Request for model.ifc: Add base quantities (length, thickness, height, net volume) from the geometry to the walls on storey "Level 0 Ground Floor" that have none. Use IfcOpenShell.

First a look at what the model holds.

```python
import ifcopenshell
import ifcopenshell.util.element
import ifcopenshell.util.unit

model = ifcopenshell.open("model.ifc")
print(model.schema)
for unit_type in ("LENGTHUNIT", "AREAUNIT", "VOLUMEUNIT"):
    print(unit_type, ifcopenshell.util.unit.calculate_unit_scale(model, unit_type))
storey = next(s for s in model.by_type("IfcBuildingStorey") if s.Name == "Level 0 Ground Floor")
walls = [e for e in ifcopenshell.util.element.get_decomposition(storey) if e.is_a("IfcWall")]
for e in sorted(walls, key=lambda e: e.id()):
    print(e.id(), e.is_a(), e.Name, list(ifcopenshell.util.element.get_psets(e, qtos_only=True)), sep=" | ")
```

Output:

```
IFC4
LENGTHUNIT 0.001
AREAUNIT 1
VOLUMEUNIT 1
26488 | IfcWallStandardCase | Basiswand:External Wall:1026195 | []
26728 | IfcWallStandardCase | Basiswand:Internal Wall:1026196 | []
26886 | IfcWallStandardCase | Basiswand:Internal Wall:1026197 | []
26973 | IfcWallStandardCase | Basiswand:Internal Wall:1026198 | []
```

```python
import ifcopenshell
import ifcopenshell.api.pset
import ifcopenshell.geom
import ifcopenshell.util.element
import ifcopenshell.util.shape
import ifcopenshell.util.unit

model = ifcopenshell.open("model.ifc")
unit_scale = ifcopenshell.util.unit.calculate_unit_scale(model)
volume_scale = ifcopenshell.util.unit.calculate_unit_scale(model, "VOLUMEUNIT")
settings = ifcopenshell.geom.settings()

storey = next(s for s in model.by_type("IfcBuildingStorey") if s.Name == "Level 0 Ground Floor")
walls = [e for e in ifcopenshell.util.element.get_decomposition(storey) if e.is_a("IfcWall")]

for e in sorted(walls, key=lambda e: e.id()):
    if ifcopenshell.util.element.get_psets(e, qtos_only=True, should_inherit=False):
        continue
    # Geometry comes back in metres, in the element's own axes.
    shape = ifcopenshell.geom.create_shape(settings, e)
    values = {
        "Length": ifcopenshell.util.shape.get_x(shape.geometry) / unit_scale,
        "Width": ifcopenshell.util.shape.get_y(shape.geometry) / unit_scale,
        "Height": ifcopenshell.util.shape.get_z(shape.geometry) / unit_scale,
        "NetVolume": ifcopenshell.util.shape.get_volume(shape.geometry) / volume_scale,
    }
    qto = ifcopenshell.api.pset.add_qto(model, product=e, name="Qto_WallBaseQuantities")
    ifcopenshell.api.pset.edit_qto(model, qto=qto, properties=values)
    print(e.id(), {k: round(v, 3) for k, v in values.items()})

model.write("model_v2.ifc")
```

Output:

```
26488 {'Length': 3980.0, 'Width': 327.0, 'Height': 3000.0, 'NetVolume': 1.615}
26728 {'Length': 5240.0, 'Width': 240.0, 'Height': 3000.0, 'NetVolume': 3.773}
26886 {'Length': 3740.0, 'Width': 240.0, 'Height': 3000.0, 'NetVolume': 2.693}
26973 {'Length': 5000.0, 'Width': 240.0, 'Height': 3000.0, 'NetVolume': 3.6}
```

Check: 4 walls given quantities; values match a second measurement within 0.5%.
